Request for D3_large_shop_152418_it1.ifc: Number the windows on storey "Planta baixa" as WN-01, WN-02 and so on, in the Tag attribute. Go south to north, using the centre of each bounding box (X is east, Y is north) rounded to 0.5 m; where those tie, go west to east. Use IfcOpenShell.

First a look at what the model holds.

```python
import ifcopenshell
import ifcopenshell.util.element
import ifcopenshell.util.placement

model = ifcopenshell.open("D3_large_shop_152418_it1.ifc")
print(model.schema)
storey = next(s for s in model.by_type("IfcBuildingStorey") if s.Name == "Planta baixa")
windows = [e for e in ifcopenshell.util.element.get_decomposition(storey) if e.is_a("IfcWindow")]
for e in sorted(windows, key=lambda e: e.id()):
    origin = ifcopenshell.util.placement.get_local_placement(e.ObjectPlacement)[:3, 3]
    print(e.id(), e.Tag, e.Name, origin.round(2) + 0.0, sep=" | ")
```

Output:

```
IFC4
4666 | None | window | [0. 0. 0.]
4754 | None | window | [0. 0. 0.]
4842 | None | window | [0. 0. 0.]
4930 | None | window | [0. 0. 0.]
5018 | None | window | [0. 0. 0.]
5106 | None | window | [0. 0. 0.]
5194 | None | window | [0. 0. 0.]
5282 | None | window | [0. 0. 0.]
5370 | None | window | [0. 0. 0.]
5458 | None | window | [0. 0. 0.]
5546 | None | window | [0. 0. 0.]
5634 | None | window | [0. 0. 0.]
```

```python
import ifcopenshell
import ifcopenshell.geom
import ifcopenshell.util.element
import ifcopenshell.util.shape

model = ifcopenshell.open("D3_large_shop_152418_it1.ifc")
settings = ifcopenshell.geom.settings()
settings.set("use-world-coords", True)


def centre(element):
    shape = ifcopenshell.geom.create_shape(settings, element)
    return ifcopenshell.util.shape.get_bbox_centroid(shape.geometry)


storey = next(s for s in model.by_type("IfcBuildingStorey") if s.Name == "Planta baixa")
windows = [e for e in ifcopenshell.util.element.get_decomposition(storey) if e.is_a("IfcWindow")]

# Insertion points can sit at a corner or the storey origin, so sort by the geometry (in metres).
centres = {e: centre(e) for e in windows}
windows.sort(key=lambda e: (round(centres[e][1] / 0.5), centres[e][0]))

for i, e in enumerate(windows, start=1):
    number = f"WN-{i:02d}"
    e.Tag = number
    print(e.id(), number)

model.write("D3_large_shop_152418_it1_rev.ifc")
```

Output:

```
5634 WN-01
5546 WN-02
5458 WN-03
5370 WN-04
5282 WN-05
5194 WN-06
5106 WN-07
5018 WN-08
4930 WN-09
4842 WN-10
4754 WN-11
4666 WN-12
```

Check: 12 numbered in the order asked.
